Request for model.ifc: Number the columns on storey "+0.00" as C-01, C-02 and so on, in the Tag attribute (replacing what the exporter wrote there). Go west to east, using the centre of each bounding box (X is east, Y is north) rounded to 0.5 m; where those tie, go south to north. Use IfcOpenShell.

First a look at what the model holds.

```python
import ifcopenshell
import ifcopenshell.util.element
import ifcopenshell.util.placement

model = ifcopenshell.open("model.ifc")
print(model.schema)
storey = next(s for s in model.by_type("IfcBuildingStorey") if s.Name == "+0.00")
columns = [e for e in ifcopenshell.util.element.get_decomposition(storey) if e.is_a("IfcColumn")]
for e in sorted(columns, key=lambda e: e.id()):
    origin = ifcopenshell.util.placement.get_local_placement(e.ObjectPlacement)[:3, 3]
    print(e.id(), e.Tag, e.Name, origin.round(2) + 0.0, sep=" | ")
```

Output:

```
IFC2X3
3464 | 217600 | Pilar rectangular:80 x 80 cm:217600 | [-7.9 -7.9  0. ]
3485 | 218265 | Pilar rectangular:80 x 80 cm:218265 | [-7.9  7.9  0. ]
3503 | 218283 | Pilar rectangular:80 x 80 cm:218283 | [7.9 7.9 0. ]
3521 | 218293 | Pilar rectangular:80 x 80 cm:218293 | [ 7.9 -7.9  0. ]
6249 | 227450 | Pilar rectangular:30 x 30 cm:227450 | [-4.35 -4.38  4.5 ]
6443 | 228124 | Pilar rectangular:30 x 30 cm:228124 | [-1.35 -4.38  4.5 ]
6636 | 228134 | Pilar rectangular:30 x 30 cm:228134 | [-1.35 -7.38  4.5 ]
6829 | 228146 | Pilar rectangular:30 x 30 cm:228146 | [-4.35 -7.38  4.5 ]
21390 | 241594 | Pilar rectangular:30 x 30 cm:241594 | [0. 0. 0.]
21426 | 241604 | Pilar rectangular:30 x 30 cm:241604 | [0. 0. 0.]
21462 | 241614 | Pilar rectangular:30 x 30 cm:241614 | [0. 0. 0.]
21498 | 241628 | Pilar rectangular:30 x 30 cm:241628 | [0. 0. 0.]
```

```python
import ifcopenshell
import ifcopenshell.geom
import ifcopenshell.util.element
import ifcopenshell.util.shape

model = ifcopenshell.open("model.ifc")
settings = ifcopenshell.geom.settings()
settings.set("use-world-coords", True)


def centre(element):
    shape = ifcopenshell.geom.create_shape(settings, element)
    return ifcopenshell.util.shape.get_bbox_centroid(shape.geometry)


storey = next(s for s in model.by_type("IfcBuildingStorey") if s.Name == "+0.00")
columns = [e for e in ifcopenshell.util.element.get_decomposition(storey) if e.is_a("IfcColumn")]

# Insertion points can sit at a corner or the storey origin, so sort by the geometry (in metres).
centres = {e: centre(e) for e in columns}
columns.sort(key=lambda e: (round(centres[e][0] / 0.5), centres[e][1]))

for i, e in enumerate(columns, start=1):
    number = f"C-{i:02d}"
    e.Tag = number
    print(e.id(), number)

model.write("model_v2.ifc")
```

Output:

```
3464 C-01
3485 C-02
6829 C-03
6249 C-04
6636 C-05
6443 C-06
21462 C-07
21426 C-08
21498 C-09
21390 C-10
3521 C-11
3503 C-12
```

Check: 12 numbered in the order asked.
